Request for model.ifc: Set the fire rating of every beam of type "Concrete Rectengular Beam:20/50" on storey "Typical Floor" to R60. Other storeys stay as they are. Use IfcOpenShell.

First a look at what the model holds.

```python
import ifcopenshell
import ifcopenshell.util.element

model = ifcopenshell.open("model.ifc")
print(model.schema)
storey = next(s for s in model.by_type("IfcBuildingStorey") if s.Name == "Typical Floor")
beams = [e for e in ifcopenshell.util.element.get_decomposition(storey) if e.is_a("IfcBeam")]
seen = {}
for e in beams:
    element_type = ifcopenshell.util.element.get_type(e)
    key = (element_type.Name if element_type != e and element_type else None, ifcopenshell.util.element.get_pset(e, "Pset_BeamCommon", "FireRating"))
    seen[key] = seen.get(key, 0) + 1
for (name, value), count in sorted(seen.items(), key=str):
    print(count, "x", name, "|", value)
```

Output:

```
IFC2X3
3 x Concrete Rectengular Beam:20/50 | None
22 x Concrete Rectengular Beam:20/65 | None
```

```python
import ifcopenshell
import ifcopenshell.api.pset
import ifcopenshell.util.element

model = ifcopenshell.open("model.ifc")

storey = next(s for s in model.by_type("IfcBuildingStorey") if s.Name == "Typical Floor")
beams = [e for e in ifcopenshell.util.element.get_decomposition(storey) if e.is_a("IfcBeam")]

count = 0
for e in beams:
    element_type = ifcopenshell.util.element.get_type(e)
    if element_type in (None, e) or element_type.Name != "Concrete Rectengular Beam:20/50":
        continue
    # add_pset returns the element's existing set when there is one.
    pset = ifcopenshell.api.pset.add_pset(model, product=e, name="Pset_BeamCommon")
    ifcopenshell.api.pset.edit_pset(model, pset=pset, properties={"FireRating": "R60"})
    count += 1

print(count, "beams updated")

model.write("model_v2.ifc")
```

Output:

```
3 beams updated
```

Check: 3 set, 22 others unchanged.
